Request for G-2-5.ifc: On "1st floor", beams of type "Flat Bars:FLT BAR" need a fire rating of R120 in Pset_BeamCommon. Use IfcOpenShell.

First a look at what the model holds.

```python
import ifcopenshell
import ifcopenshell.util.element

model = ifcopenshell.open("G-2-5.ifc")
print(model.schema)
storey = next(s for s in model.by_type("IfcBuildingStorey") if s.Name == "1st floor")
beams = [e for e in ifcopenshell.util.element.get_decomposition(storey) if e.is_a("IfcBeam")]
seen = {}
for e in beams:
    element_type = ifcopenshell.util.element.get_type(e)
    key = (element_type.Name if element_type != e and element_type else None, ifcopenshell.util.element.get_pset(e, "Pset_BeamCommon", "FireRating"))
    seen[key] = seen.get(key, 0) + 1
for (name, value), count in sorted(seen.items(), key=str):
    print(count, "x", name, "|", value)
```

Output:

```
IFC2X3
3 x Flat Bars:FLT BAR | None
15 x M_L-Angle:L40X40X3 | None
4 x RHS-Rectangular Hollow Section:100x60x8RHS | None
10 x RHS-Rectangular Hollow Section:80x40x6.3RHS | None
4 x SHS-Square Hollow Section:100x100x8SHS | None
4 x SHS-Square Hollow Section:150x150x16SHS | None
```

```python
import ifcopenshell
import ifcopenshell.api.pset
import ifcopenshell.util.element

model = ifcopenshell.open("G-2-5.ifc")

storey = next(s for s in model.by_type("IfcBuildingStorey") if s.Name == "1st floor")
beams = [e for e in ifcopenshell.util.element.get_decomposition(storey) if e.is_a("IfcBeam")]

count = 0
for e in beams:
    element_type = ifcopenshell.util.element.get_type(e)
    if element_type in (None, e) or element_type.Name != "Flat Bars:FLT BAR":
        continue
    # add_pset returns the element's existing set when there is one.
    pset = ifcopenshell.api.pset.add_pset(model, product=e, name="Pset_BeamCommon")
    ifcopenshell.api.pset.edit_pset(model, pset=pset, properties={"FireRating": "R120"})
    count += 1

print(count, "beams updated")

model.write("G-2-5_updated.ifc")
```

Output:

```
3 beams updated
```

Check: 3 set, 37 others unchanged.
